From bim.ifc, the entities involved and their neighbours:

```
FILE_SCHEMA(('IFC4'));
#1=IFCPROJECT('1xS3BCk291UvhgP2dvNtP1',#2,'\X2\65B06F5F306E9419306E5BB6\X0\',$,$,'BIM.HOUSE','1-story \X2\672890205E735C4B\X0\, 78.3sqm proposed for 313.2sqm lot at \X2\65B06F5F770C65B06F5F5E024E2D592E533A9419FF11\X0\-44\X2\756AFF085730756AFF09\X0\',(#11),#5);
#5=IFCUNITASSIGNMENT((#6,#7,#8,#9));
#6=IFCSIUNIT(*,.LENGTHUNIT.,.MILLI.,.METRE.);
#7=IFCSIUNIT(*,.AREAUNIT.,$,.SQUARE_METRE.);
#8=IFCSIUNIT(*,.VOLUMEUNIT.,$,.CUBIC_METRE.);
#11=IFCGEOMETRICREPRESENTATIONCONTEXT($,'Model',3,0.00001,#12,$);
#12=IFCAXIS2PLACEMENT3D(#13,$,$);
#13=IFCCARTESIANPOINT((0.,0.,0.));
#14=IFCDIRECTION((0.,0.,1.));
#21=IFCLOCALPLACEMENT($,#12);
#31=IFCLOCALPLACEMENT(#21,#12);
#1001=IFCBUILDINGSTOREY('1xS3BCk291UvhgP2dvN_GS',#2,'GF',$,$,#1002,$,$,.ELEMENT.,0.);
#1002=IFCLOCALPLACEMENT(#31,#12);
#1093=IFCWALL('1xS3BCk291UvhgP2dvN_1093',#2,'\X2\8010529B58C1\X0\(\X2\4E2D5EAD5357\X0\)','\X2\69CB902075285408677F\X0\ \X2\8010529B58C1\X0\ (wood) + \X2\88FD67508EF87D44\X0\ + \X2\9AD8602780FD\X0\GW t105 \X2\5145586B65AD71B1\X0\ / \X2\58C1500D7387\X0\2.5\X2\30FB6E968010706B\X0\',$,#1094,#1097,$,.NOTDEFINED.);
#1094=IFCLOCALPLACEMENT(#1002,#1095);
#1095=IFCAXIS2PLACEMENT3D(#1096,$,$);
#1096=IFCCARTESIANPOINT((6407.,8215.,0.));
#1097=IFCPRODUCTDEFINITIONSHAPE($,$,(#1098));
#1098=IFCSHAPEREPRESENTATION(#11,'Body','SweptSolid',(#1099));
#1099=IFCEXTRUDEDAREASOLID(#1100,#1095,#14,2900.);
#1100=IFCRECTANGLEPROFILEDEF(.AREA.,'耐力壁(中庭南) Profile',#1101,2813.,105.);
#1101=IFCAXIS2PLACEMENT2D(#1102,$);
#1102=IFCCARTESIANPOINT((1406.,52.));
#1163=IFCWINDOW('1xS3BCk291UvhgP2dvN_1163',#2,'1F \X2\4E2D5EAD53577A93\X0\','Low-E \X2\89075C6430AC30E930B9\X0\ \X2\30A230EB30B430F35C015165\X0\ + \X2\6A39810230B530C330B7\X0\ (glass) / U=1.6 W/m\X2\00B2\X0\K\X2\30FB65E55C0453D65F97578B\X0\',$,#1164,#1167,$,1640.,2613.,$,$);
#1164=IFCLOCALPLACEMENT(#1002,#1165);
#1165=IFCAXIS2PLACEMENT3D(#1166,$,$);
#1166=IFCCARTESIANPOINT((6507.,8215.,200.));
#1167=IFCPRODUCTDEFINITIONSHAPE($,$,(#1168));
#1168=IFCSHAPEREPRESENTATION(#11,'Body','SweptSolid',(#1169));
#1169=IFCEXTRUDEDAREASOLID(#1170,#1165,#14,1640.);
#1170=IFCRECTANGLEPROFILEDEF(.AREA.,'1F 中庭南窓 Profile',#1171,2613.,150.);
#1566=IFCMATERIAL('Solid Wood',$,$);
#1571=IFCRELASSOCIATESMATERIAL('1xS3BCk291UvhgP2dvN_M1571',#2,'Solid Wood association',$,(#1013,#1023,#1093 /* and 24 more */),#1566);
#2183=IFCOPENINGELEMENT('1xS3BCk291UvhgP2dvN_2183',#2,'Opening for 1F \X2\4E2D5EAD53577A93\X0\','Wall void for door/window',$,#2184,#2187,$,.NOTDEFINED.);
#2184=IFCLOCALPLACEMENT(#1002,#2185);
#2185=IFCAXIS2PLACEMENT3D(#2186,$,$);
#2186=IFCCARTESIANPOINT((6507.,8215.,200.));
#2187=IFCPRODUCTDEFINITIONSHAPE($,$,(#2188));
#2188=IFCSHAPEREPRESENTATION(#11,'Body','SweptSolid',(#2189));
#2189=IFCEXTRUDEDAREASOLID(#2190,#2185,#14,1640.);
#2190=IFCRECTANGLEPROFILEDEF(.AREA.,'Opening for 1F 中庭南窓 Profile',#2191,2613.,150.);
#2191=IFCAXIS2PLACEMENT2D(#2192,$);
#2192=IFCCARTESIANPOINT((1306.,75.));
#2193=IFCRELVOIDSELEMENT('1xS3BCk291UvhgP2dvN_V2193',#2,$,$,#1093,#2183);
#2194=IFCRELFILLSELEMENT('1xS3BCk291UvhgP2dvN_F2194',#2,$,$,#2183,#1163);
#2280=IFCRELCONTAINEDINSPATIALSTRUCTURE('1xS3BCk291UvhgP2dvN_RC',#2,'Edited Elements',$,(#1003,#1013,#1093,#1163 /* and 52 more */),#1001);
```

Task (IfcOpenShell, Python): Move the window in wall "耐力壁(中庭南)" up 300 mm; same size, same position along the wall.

```python
import numpy as np
import ifcopenshell
import ifcopenshell.api.geometry
import ifcopenshell.util.placement
import ifcopenshell.util.unit

model = ifcopenshell.open("bim.ifc")
unit_scale = ifcopenshell.util.unit.calculate_unit_scale(model)

window = model.by_id(1163)
opening = window.FillsVoids[0].RelatingOpeningElement
dz = 0.3 / unit_scale

shift = np.array([0.0, 0.0, dz])
# The window is not placed relative to its opening, so move both.
for product in (opening, window):
    matrix = ifcopenshell.util.placement.get_local_placement(product.ObjectPlacement)
    matrix[:3, 3] += shift
    ifcopenshell.api.geometry.edit_object_placement(model, product=product, matrix=matrix, is_si=False)

print(f"moved by {dz * unit_scale:+.3f} m")

model.write("bim_rev.ifc")
```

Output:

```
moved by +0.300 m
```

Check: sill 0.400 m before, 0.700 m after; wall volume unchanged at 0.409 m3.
